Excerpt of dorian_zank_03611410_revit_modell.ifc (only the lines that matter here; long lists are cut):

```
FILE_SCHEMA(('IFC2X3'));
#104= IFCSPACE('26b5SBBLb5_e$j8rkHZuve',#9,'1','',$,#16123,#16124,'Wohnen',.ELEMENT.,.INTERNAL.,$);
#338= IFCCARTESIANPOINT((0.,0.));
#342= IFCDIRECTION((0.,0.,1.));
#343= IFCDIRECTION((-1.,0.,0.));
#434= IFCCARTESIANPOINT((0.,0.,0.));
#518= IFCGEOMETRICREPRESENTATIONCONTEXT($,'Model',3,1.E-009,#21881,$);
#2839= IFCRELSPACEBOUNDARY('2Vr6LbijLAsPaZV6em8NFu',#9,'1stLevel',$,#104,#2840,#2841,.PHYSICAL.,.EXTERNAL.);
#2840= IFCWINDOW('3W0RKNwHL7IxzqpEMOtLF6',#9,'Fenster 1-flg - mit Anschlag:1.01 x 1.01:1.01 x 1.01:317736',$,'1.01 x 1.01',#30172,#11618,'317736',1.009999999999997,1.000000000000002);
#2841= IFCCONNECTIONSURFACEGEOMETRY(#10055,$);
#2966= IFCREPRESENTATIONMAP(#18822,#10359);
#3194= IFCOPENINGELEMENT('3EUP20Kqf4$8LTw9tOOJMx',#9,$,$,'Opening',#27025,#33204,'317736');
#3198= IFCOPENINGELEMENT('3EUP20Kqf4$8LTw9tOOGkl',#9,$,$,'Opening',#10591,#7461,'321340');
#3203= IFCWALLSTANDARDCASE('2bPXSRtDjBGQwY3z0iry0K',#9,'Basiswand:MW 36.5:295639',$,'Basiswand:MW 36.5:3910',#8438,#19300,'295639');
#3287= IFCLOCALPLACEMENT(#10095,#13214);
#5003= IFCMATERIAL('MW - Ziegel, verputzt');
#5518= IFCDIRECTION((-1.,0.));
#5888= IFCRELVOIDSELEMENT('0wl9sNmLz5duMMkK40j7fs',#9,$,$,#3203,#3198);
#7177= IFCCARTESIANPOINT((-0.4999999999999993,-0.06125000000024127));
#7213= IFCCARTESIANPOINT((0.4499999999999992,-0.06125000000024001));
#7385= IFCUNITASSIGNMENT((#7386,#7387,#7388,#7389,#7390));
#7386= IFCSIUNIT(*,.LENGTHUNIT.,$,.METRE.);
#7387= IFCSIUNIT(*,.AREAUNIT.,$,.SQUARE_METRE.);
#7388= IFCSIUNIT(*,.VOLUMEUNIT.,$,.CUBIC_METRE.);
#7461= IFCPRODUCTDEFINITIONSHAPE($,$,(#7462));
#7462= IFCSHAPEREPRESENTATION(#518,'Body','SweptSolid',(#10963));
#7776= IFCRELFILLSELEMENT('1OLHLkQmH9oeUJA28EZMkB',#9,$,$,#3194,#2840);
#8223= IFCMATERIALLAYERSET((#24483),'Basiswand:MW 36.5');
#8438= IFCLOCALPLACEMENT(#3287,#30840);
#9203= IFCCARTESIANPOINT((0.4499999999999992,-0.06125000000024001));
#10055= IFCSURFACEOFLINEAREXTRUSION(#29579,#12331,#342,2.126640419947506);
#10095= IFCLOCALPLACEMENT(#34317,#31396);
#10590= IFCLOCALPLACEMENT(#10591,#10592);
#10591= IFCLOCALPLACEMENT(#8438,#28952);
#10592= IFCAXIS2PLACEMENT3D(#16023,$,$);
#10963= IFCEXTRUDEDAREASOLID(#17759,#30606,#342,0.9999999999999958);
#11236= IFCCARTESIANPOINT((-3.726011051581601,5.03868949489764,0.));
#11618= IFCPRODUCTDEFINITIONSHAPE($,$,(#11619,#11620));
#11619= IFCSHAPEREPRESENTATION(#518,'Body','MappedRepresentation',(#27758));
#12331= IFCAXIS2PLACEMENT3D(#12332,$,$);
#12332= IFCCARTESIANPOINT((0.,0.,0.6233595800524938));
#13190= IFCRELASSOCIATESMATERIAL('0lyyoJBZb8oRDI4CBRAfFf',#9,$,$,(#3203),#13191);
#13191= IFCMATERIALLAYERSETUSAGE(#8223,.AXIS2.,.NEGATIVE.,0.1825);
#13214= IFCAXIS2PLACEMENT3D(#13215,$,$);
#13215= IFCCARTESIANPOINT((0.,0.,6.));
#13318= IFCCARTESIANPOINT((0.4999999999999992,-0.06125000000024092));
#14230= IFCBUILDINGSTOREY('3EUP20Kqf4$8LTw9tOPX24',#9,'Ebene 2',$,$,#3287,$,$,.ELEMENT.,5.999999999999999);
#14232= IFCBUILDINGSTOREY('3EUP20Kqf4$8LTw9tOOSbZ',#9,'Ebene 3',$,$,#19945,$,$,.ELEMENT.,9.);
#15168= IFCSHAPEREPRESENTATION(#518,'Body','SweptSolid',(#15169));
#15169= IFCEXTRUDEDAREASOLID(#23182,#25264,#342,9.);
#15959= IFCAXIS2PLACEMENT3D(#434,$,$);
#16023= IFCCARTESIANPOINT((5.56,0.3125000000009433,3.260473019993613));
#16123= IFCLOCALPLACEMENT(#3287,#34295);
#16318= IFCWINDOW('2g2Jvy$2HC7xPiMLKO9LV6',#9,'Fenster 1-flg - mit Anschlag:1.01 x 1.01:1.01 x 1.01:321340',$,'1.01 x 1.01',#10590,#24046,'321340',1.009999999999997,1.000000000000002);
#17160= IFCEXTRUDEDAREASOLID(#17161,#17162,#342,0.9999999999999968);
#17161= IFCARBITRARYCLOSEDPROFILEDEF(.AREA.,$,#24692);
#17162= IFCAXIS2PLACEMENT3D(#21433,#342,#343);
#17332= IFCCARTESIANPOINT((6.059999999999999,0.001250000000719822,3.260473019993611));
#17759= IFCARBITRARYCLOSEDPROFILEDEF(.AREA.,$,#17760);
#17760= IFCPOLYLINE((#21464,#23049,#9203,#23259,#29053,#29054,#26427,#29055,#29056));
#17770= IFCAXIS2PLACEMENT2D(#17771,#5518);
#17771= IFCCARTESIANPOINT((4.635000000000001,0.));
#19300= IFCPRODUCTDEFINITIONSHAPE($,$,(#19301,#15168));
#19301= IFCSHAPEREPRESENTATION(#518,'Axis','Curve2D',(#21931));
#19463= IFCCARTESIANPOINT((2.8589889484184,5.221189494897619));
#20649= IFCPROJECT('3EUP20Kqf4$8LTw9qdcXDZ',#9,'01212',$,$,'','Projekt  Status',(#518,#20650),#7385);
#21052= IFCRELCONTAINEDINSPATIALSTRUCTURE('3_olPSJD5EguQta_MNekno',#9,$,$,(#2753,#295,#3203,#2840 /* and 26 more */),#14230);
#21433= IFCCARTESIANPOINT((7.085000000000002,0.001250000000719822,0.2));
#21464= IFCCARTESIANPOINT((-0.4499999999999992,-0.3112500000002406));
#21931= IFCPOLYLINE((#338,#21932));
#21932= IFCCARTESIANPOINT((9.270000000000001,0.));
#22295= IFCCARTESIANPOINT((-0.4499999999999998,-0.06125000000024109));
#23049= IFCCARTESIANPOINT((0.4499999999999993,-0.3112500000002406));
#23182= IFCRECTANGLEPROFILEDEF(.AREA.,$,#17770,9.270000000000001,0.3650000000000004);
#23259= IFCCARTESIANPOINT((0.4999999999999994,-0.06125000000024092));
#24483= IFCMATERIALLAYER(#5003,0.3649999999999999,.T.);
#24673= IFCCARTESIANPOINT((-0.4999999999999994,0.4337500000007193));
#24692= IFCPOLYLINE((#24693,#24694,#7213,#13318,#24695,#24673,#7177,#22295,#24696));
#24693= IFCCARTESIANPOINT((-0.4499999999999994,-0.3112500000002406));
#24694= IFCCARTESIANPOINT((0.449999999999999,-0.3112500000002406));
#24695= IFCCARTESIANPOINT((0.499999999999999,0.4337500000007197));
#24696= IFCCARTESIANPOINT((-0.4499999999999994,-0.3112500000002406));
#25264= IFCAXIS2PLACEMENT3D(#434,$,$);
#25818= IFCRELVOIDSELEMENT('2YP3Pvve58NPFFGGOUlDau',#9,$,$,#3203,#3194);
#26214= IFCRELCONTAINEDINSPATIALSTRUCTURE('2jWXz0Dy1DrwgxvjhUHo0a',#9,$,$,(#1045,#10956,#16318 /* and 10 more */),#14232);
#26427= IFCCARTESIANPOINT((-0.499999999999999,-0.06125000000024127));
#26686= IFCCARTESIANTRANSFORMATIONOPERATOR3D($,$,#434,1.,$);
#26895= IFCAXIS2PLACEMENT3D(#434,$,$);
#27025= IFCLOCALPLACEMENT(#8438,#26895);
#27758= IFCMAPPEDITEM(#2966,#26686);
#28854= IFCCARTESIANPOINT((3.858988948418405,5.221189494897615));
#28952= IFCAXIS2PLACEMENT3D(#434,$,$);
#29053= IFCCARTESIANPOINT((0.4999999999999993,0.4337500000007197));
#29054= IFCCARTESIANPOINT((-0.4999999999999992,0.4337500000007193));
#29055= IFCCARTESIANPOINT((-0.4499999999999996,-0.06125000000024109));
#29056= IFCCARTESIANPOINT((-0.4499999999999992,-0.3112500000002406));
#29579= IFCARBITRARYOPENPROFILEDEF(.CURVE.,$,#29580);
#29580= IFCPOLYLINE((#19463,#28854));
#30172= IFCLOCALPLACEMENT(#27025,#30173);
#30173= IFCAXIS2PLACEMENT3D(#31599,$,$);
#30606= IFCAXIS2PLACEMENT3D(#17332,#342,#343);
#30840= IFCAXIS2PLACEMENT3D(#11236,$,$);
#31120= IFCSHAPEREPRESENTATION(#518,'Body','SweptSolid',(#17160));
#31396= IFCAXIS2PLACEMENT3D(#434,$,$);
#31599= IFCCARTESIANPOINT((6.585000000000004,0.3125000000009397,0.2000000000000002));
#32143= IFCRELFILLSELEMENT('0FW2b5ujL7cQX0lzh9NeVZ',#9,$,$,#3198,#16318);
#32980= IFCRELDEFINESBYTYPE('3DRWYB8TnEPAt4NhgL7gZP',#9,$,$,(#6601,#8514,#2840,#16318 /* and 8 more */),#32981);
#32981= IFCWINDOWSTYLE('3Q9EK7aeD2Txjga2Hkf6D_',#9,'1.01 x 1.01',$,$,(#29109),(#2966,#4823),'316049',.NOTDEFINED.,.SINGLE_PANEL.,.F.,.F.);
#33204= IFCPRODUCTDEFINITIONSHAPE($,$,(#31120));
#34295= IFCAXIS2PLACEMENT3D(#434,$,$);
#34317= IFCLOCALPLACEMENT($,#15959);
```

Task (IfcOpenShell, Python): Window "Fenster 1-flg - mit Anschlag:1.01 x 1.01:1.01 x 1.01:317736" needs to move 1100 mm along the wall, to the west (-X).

```python
import numpy as np
import ifcopenshell
import ifcopenshell.api.geometry
import ifcopenshell.util.placement

model = ifcopenshell.open("dorian_zank_03611410_revit_modell.ifc")

window = model.by_guid("3W0RKNwHL7IxzqpEMOtLF6")
opening = window.FillsVoids[0].RelatingOpeningElement
wall = opening.VoidsElements[0].RelatingBuildingElement

wall_matrix = ifcopenshell.util.placement.get_local_placement(wall.ObjectPlacement)
shift = wall_matrix[:3, 0] * -1.1
before = ifcopenshell.util.placement.get_local_placement(window.ObjectPlacement)[:3, 3].copy()

# The window is placed relative to its opening, so it follows when the opening moves.
matrix = ifcopenshell.util.placement.get_local_placement(opening.ObjectPlacement)
matrix[:3, 3] += shift
ifcopenshell.api.geometry.edit_object_placement(
    model, product=opening, matrix=matrix, is_si=False, should_transform_children=True
)

# Space boundary surfaces are stored in each space's coordinates; move them too.
for rel in window.ProvidesBoundaries:
    if not rel.ConnectionGeometry:
        continue
    surface = rel.ConnectionGeometry.SurfaceOnRelatingElement
    space_matrix = ifcopenshell.util.placement.get_local_placement(rel.RelatingSpace.ObjectPlacement)
    point = np.array(surface.Position.Location.Coordinates) + space_matrix[:3, :3].T @ shift
    surface.Position = model.createIfcAxis2Placement3D(
        model.createIfcCartesianPoint(point.tolist()), surface.Position.Axis, surface.Position.RefDirection
    )

after = ifcopenshell.util.placement.get_local_placement(window.ObjectPlacement)[:3, 3]
print("window moved by", (after - before).round(3) + 0.0)

model.write("dorian_zank_03611410_revit_modell_edited.ifc")
```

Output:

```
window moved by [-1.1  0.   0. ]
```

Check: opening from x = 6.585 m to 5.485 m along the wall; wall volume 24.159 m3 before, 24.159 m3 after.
